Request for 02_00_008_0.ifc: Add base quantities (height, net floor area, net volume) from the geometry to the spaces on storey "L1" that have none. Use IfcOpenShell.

First a look at what the model holds.

```python
import ifcopenshell
import ifcopenshell.util.element
import ifcopenshell.util.unit

model = ifcopenshell.open("02_00_008_0.ifc")
print(model.schema)
for unit_type in ("LENGTHUNIT", "AREAUNIT", "VOLUMEUNIT"):
    print(unit_type, ifcopenshell.util.unit.calculate_unit_scale(model, unit_type))
storey = next(s for s in model.by_type("IfcBuildingStorey") if s.Name == "L1")
spaces = [e for e in ifcopenshell.util.element.get_decomposition(storey) if e.is_a("IfcSpace")]
for e in sorted(spaces, key=lambda e: e.id()):
    print(e.id(), e.is_a(), e.Name, list(ifcopenshell.util.element.get_psets(e, qtos_only=True)), sep=" | ")
```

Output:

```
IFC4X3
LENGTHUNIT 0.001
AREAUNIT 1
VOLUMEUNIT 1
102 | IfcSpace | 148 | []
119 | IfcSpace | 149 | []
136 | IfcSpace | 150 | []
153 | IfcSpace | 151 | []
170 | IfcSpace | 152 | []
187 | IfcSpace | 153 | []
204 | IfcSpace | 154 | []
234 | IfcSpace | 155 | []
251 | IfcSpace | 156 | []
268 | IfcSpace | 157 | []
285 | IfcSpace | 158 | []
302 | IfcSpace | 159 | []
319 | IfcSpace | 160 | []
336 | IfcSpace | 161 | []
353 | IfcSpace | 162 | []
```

```python
import ifcopenshell
import ifcopenshell.api.pset
import ifcopenshell.geom
import ifcopenshell.util.element
import ifcopenshell.util.shape
import ifcopenshell.util.unit

model = ifcopenshell.open("02_00_008_0.ifc")
unit_scale = ifcopenshell.util.unit.calculate_unit_scale(model)
area_scale = ifcopenshell.util.unit.calculate_unit_scale(model, "AREAUNIT")
volume_scale = ifcopenshell.util.unit.calculate_unit_scale(model, "VOLUMEUNIT")
settings = ifcopenshell.geom.settings()

storey = next(s for s in model.by_type("IfcBuildingStorey") if s.Name == "L1")
spaces = [e for e in ifcopenshell.util.element.get_decomposition(storey) if e.is_a("IfcSpace")]

for e in sorted(spaces, key=lambda e: e.id()):
    if ifcopenshell.util.element.get_psets(e, qtos_only=True, should_inherit=False):
        continue
    # Geometry comes back in metres, in the element's own axes.
    shape = ifcopenshell.geom.create_shape(settings, e)
    values = {
        "Height": ifcopenshell.util.shape.get_z(shape.geometry) / unit_scale,
        "NetFloorArea": ifcopenshell.util.shape.get_footprint_area(shape.geometry) / area_scale,
        "NetVolume": ifcopenshell.util.shape.get_volume(shape.geometry) / volume_scale,
    }
    qto = ifcopenshell.api.pset.add_qto(model, product=e, name="Qto_SpaceBaseQuantities")
    ifcopenshell.api.pset.edit_qto(model, qto=qto, properties=values)
    print(e.id(), {k: round(v, 3) for k, v in values.items()})

model.write("02_00_008_0_edited.ifc")
```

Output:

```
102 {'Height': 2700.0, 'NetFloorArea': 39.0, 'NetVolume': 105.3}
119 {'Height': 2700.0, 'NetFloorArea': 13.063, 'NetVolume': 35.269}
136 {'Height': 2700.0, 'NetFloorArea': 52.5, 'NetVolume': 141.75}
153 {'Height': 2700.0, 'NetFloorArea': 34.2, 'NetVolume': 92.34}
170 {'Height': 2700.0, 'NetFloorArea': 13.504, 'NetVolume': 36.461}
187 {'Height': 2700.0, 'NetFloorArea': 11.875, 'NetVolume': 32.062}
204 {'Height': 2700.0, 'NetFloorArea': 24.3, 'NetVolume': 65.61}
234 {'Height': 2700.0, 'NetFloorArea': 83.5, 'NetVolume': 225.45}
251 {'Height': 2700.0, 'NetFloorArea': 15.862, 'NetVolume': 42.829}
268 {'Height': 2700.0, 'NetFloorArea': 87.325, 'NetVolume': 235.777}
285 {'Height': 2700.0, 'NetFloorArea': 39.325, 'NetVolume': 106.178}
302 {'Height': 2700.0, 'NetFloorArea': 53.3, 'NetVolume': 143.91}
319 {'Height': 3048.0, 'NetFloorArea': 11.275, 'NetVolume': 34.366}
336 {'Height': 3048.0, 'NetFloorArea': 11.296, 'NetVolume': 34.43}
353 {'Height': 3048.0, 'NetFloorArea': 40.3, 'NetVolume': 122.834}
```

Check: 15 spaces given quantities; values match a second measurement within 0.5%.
